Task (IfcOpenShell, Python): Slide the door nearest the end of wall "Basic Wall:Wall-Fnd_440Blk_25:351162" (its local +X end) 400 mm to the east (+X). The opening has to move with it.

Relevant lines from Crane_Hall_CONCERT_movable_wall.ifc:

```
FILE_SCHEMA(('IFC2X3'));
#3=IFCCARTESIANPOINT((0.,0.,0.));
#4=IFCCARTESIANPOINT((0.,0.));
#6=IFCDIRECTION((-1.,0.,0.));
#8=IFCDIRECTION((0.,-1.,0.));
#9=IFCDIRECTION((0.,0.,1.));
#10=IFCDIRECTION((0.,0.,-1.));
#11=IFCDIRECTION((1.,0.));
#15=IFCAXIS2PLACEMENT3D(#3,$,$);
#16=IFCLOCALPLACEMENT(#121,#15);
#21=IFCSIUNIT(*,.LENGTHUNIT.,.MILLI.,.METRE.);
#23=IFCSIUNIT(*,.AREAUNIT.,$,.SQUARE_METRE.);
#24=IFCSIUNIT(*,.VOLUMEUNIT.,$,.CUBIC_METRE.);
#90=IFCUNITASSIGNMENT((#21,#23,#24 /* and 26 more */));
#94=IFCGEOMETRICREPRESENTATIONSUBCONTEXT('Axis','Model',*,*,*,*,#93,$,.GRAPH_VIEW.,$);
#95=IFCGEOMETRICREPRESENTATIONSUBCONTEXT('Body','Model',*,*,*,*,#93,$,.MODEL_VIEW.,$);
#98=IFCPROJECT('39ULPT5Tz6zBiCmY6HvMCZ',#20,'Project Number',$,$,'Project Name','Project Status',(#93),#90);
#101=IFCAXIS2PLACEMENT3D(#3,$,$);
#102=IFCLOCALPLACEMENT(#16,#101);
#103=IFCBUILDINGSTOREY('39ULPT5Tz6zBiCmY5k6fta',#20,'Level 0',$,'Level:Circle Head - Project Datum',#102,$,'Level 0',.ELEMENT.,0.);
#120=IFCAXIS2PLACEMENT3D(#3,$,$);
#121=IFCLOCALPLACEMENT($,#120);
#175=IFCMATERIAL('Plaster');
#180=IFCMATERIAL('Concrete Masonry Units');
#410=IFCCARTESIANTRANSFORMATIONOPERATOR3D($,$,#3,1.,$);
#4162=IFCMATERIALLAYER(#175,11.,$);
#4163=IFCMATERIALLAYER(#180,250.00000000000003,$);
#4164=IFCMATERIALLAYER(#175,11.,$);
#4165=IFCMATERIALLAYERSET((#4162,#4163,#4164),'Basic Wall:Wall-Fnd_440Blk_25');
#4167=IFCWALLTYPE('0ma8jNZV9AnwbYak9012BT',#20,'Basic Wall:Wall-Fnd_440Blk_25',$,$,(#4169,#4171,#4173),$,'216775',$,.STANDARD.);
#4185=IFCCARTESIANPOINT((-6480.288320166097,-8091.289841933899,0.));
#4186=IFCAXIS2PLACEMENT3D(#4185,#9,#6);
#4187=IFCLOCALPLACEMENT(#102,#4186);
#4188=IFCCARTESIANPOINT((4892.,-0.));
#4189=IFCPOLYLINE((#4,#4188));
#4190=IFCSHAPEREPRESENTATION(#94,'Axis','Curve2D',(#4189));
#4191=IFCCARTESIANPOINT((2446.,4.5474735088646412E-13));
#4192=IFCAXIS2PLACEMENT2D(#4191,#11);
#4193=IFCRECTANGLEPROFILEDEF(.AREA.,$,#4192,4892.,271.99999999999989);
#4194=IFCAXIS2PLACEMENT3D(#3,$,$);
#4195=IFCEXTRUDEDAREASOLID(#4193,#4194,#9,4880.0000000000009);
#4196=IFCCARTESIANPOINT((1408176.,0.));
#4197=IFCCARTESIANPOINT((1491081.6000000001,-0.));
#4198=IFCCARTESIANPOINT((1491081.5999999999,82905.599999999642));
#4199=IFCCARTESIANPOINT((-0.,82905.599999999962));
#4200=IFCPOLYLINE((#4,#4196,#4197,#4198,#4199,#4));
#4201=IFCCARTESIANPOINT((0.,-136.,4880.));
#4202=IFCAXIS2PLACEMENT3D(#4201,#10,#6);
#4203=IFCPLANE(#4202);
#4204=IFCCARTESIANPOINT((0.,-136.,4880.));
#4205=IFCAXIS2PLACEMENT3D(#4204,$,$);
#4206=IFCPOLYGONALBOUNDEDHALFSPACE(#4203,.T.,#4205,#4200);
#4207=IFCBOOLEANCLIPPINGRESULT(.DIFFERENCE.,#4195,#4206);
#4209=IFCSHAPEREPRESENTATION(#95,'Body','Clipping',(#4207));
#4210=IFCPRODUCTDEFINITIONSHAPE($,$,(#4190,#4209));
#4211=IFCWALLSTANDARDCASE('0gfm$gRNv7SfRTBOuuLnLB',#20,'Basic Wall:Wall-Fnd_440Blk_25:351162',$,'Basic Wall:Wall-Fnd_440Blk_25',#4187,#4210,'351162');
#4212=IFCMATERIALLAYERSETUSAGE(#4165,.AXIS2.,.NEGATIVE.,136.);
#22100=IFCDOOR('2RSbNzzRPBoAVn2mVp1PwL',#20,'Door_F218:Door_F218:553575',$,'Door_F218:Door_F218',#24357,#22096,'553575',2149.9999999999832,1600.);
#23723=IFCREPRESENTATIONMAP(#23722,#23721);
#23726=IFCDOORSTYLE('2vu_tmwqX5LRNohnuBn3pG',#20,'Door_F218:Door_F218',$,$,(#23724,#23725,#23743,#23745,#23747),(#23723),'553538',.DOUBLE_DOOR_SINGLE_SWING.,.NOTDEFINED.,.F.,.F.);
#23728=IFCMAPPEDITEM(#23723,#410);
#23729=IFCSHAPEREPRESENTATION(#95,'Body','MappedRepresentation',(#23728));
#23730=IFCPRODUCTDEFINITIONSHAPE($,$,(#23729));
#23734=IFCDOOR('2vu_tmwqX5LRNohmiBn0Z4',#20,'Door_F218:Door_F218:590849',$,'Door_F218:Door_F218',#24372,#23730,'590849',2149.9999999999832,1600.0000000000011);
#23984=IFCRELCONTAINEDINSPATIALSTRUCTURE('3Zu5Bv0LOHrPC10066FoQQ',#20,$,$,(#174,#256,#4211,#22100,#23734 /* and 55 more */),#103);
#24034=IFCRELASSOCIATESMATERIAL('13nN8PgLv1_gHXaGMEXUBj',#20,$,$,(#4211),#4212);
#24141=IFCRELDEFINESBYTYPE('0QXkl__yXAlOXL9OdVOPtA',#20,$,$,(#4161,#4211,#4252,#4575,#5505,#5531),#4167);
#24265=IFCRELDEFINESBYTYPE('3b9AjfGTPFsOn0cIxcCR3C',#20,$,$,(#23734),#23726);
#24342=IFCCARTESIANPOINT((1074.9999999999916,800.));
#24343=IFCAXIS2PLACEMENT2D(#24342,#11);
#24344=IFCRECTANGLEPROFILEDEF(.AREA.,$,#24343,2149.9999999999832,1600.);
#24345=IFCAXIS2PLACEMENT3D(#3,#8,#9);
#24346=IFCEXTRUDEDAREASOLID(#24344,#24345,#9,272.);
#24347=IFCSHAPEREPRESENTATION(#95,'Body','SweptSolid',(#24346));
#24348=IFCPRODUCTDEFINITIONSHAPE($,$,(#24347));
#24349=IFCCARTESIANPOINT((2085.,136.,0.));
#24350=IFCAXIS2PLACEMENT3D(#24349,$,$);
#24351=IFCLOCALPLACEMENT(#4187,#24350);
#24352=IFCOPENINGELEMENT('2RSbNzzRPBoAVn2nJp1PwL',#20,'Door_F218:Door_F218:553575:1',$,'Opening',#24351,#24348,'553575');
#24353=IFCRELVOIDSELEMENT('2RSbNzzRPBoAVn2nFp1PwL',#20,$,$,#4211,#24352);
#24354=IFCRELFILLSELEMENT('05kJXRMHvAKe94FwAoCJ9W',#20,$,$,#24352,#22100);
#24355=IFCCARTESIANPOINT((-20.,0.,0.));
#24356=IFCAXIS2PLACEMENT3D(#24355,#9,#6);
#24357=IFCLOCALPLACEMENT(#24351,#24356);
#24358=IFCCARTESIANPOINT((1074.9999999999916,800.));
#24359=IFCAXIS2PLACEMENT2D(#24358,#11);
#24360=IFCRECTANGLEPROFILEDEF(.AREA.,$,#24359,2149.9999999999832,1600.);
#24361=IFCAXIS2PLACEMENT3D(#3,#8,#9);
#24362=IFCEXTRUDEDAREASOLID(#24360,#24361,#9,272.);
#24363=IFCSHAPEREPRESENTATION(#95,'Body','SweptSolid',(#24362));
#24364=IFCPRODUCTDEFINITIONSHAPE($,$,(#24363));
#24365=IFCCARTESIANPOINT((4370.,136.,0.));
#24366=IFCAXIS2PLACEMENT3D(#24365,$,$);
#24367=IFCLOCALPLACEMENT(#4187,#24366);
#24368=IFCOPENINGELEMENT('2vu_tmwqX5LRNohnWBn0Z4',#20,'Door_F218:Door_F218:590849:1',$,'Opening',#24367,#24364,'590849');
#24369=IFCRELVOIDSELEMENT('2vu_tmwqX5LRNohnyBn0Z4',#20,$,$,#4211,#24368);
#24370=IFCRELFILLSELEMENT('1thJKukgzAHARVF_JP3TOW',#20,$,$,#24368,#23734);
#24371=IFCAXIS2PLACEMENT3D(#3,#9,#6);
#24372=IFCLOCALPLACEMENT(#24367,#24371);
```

```python
import ifcopenshell
import ifcopenshell.api.geometry
import ifcopenshell.util.placement
import ifcopenshell.util.unit

model = ifcopenshell.open("Crane_Hall_CONCERT_movable_wall.ifc")
unit_scale = ifcopenshell.util.unit.calculate_unit_scale(model)

door = model.by_guid("2vu_tmwqX5LRNohmiBn0Z4")
opening = door.FillsVoids[0].RelatingOpeningElement
wall = opening.VoidsElements[0].RelatingBuildingElement

wall_matrix = ifcopenshell.util.placement.get_local_placement(wall.ObjectPlacement)
shift = wall_matrix[:3, 0] * -0.4 / unit_scale
before = ifcopenshell.util.placement.get_local_placement(door.ObjectPlacement)[:3, 3].copy()

# The door is placed relative to its opening, so it follows when the opening moves.
matrix = ifcopenshell.util.placement.get_local_placement(opening.ObjectPlacement)
matrix[:3, 3] += shift
ifcopenshell.api.geometry.edit_object_placement(
    model, product=opening, matrix=matrix, is_si=False, should_transform_children=True
)

after = ifcopenshell.util.placement.get_local_placement(door.ObjectPlacement)[:3, 3]
print("door moved by", (after - before).round(3) + 0.0)

model.write("Crane_Hall_CONCERT_movable_wall_rev.ifc")
```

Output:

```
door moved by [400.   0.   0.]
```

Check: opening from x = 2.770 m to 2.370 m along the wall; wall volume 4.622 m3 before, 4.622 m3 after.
